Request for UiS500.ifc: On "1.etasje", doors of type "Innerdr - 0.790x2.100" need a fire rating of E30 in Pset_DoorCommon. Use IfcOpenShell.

First a look at what the model holds.

```python
import ifcopenshell
import ifcopenshell.util.element

model = ifcopenshell.open("UiS500.ifc")
print(model.schema)
storey = next(s for s in model.by_type("IfcBuildingStorey") if s.Name == "1.etasje")
doors = [e for e in ifcopenshell.util.element.get_decomposition(storey) if e.is_a("IfcDoor")]
seen = {}
for e in doors:
    element_type = ifcopenshell.util.element.get_type(e)
    key = (element_type.Name if element_type != e and element_type else None, ifcopenshell.util.element.get_pset(e, "Pset_DoorCommon", "FireRating"))
    seen[key] = seen.get(key, 0) + 1
for (name, value), count in sorted(seen.items(), key=str):
    print(count, "x", name, "|", value)
```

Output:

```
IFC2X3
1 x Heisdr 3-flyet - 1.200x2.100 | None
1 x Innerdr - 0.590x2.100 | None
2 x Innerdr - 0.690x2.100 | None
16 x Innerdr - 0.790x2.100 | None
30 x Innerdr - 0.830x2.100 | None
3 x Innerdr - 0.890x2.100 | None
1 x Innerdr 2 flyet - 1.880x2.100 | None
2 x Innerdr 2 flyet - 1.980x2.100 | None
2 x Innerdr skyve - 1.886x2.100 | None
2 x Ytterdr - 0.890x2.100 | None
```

```python
import ifcopenshell
import ifcopenshell.api.pset
import ifcopenshell.util.element

model = ifcopenshell.open("UiS500.ifc")

storey = next(s for s in model.by_type("IfcBuildingStorey") if s.Name == "1.etasje")
doors = [e for e in ifcopenshell.util.element.get_decomposition(storey) if e.is_a("IfcDoor")]

count = 0
for e in doors:
    element_type = ifcopenshell.util.element.get_type(e)
    if element_type in (None, e) or element_type.Name != 'Innerd\x9br - 0.790x2.100':
        continue
    # add_pset returns the element's existing set when there is one.
    pset = ifcopenshell.api.pset.add_pset(model, product=e, name="Pset_DoorCommon")
    ifcopenshell.api.pset.edit_pset(model, pset=pset, properties={"FireRating": "E30"})
    count += 1

print(count, "doors updated")

model.write("UiS500-out.ifc")
```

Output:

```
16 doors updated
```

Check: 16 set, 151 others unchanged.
